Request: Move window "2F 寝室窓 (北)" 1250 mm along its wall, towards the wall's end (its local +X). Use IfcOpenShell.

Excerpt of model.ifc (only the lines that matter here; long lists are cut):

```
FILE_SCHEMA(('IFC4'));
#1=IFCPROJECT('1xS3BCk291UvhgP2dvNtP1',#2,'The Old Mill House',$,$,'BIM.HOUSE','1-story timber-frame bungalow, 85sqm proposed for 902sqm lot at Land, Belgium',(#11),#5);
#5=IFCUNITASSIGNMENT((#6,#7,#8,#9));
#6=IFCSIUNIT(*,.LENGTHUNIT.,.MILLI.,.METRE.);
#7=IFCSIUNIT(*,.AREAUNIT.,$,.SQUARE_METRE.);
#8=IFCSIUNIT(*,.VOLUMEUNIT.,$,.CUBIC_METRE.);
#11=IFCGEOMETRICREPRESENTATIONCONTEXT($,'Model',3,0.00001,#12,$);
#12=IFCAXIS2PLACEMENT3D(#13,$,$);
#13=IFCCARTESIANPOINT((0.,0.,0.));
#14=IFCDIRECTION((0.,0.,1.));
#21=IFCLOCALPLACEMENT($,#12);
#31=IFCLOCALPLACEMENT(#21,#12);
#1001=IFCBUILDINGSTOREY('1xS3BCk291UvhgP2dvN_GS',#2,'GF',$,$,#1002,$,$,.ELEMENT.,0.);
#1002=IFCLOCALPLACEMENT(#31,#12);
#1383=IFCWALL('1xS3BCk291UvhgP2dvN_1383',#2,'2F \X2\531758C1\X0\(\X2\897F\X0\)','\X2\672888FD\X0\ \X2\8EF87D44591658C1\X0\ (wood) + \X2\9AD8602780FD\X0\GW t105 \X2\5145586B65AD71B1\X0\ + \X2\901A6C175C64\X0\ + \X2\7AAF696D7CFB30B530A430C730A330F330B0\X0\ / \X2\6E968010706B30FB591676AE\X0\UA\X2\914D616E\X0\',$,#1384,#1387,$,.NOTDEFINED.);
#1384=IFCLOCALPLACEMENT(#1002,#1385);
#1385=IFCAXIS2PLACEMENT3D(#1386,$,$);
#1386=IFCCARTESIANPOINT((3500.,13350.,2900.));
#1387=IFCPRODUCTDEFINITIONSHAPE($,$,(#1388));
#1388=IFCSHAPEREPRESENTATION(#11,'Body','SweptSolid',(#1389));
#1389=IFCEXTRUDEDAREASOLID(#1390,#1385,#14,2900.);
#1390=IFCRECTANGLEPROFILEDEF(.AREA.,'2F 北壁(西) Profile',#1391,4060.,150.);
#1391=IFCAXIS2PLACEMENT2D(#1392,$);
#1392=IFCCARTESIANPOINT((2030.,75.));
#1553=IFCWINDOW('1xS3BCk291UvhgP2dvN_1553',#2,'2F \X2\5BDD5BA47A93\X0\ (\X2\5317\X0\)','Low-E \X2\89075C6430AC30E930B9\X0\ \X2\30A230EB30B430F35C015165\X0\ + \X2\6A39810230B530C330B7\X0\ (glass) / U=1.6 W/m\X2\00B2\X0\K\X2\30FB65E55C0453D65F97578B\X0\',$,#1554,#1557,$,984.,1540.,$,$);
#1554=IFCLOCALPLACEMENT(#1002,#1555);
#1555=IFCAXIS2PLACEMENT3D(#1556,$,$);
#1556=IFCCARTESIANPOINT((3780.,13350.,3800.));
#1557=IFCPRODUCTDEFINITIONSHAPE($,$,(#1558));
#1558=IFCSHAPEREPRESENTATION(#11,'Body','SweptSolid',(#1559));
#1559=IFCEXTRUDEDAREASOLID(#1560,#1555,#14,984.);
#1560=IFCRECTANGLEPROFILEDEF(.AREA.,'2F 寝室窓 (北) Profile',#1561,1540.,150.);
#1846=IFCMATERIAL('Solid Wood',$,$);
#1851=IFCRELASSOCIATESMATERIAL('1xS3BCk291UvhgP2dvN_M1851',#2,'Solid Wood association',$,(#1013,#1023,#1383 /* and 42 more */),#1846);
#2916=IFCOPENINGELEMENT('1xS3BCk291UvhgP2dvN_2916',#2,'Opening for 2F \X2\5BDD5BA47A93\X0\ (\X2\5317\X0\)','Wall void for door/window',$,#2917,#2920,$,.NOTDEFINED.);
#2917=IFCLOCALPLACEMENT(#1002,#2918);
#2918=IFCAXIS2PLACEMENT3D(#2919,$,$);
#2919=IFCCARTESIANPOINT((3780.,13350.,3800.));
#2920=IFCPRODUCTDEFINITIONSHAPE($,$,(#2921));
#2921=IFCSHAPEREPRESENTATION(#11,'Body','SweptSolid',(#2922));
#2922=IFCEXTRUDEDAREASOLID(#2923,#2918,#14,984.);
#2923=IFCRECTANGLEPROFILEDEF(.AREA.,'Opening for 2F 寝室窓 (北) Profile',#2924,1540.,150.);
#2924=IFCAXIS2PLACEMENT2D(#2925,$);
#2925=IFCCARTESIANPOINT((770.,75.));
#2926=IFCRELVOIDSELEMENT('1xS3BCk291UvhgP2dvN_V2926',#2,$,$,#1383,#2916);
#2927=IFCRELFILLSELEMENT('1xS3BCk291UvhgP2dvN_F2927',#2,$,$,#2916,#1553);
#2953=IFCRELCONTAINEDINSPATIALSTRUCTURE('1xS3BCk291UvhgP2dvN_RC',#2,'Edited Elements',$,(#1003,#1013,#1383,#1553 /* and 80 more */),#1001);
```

```python
import ifcopenshell
import ifcopenshell.api.geometry
import ifcopenshell.util.placement
import ifcopenshell.util.unit

model = ifcopenshell.open("model.ifc")
unit_scale = ifcopenshell.util.unit.calculate_unit_scale(model)

window = model.by_guid("1xS3BCk291UvhgP2dvN_1553")
opening = window.FillsVoids[0].RelatingOpeningElement
wall = opening.VoidsElements[0].RelatingBuildingElement

wall_matrix = ifcopenshell.util.placement.get_local_placement(wall.ObjectPlacement)
shift = wall_matrix[:3, 0] * 1.25 / unit_scale
before = ifcopenshell.util.placement.get_local_placement(window.ObjectPlacement)[:3, 3].copy()

# The window is not placed relative to its opening, so move both.
for product in (opening, window):
    matrix = ifcopenshell.util.placement.get_local_placement(product.ObjectPlacement)
    matrix[:3, 3] += shift
    ifcopenshell.api.geometry.edit_object_placement(model, product=product, matrix=matrix, is_si=False)

after = ifcopenshell.util.placement.get_local_placement(window.ObjectPlacement)[:3, 3]
print("window moved by", (after - before).round(3) + 0.0)

model.write("model_updated.ifc")
```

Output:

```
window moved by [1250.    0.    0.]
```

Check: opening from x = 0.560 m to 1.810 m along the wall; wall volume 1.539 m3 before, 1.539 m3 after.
